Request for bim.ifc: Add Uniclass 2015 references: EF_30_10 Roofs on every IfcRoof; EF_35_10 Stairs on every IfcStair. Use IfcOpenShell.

First a look at what the model holds.

```python
import ifcopenshell

model = ifcopenshell.open("bim.ifc")
print(model.schema)
print("classifications:", [c.Name for c in model.by_type("IfcClassification")])
for ifc_class in ("IfcDoor", "IfcRoof", "IfcStair", "IfcWall", "IfcWindow"):
    print(ifc_class, len(model.by_type(ifc_class)))
```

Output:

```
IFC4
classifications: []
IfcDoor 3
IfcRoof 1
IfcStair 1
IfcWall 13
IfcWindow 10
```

```python
import ifcopenshell
import ifcopenshell.api.classification

model = ifcopenshell.open("bim.ifc")

system = ifcopenshell.api.classification.add_classification(model, classification="Uniclass 2015")

codes = {
    "IfcRoof": ("EF_30_10", "Roofs"),
    "IfcStair": ("EF_35_10", "Stairs"),
}
for ifc_class, (code, name) in codes.items():
    products = model.by_type(ifc_class)
    ifcopenshell.api.classification.add_reference(
        model, products=products, classification=system, identification=code, name=name
    )
    print(code, len(products))

model.write("bim_rev.ifc")
```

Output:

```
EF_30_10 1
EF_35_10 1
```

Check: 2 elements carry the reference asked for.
